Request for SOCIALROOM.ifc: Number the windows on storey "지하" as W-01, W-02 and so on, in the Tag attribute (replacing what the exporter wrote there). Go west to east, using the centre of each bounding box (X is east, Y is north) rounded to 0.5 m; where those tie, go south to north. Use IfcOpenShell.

First a look at what the model holds.

```python
import ifcopenshell
import ifcopenshell.util.element
import ifcopenshell.util.placement

model = ifcopenshell.open("SOCIALROOM.ifc")
print(model.schema)
storey = next(s for s in model.by_type("IfcBuildingStorey") if s.Name == "지하")
windows = [e for e in ifcopenshell.util.element.get_decomposition(storey) if e.is_a("IfcWindow")]
for e in sorted(windows, key=lambda e: e.id()):
    origin = ifcopenshell.util.placement.get_local_placement(e.ObjectPlacement)[:3, 3]
    print(e.id(), e.Tag, e.Name, origin.round(2) + 0.0, sep=" | ")
```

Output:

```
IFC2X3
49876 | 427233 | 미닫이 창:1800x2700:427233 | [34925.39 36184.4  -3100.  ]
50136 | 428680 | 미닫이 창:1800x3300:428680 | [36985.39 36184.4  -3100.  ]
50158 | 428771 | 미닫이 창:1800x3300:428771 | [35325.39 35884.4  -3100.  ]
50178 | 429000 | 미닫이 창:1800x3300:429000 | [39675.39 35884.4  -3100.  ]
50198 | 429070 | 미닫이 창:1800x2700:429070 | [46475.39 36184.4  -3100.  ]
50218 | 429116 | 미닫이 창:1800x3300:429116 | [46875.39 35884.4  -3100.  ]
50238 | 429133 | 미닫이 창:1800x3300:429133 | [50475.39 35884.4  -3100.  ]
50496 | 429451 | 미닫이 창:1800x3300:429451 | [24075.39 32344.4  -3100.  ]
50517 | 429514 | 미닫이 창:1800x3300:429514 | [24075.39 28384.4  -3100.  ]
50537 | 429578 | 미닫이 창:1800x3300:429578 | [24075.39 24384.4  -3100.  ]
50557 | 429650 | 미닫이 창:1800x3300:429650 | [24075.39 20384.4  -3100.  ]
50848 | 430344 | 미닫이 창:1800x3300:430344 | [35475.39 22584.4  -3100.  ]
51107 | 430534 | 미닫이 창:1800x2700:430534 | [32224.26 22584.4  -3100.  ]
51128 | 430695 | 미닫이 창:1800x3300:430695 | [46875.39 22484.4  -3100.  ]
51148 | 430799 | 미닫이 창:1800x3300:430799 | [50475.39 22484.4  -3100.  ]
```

```python
import ifcopenshell
import ifcopenshell.geom
import ifcopenshell.util.element
import ifcopenshell.util.shape

model = ifcopenshell.open("SOCIALROOM.ifc")
settings = ifcopenshell.geom.settings()
settings.set("use-world-coords", True)


def centre(element):
    shape = ifcopenshell.geom.create_shape(settings, element)
    return ifcopenshell.util.shape.get_bbox_centroid(shape.geometry)


storey = next(s for s in model.by_type("IfcBuildingStorey") if s.Name == "지하")
windows = [e for e in ifcopenshell.util.element.get_decomposition(storey) if e.is_a("IfcWindow")]

# Insertion points can sit at a corner or the storey origin, so sort by the geometry (in metres).
centres = {e: centre(e) for e in windows}
windows.sort(key=lambda e: (round(centres[e][0] / 0.5), centres[e][1]))

for i, e in enumerate(windows, start=1):
    number = f"W-{i:02d}"
    e.Tag = number
    print(e.id(), number)

model.write("SOCIALROOM_updated.ifc")
```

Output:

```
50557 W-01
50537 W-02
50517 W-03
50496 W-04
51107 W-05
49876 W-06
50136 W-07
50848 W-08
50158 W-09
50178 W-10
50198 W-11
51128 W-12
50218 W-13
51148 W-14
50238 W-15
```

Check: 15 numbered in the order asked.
